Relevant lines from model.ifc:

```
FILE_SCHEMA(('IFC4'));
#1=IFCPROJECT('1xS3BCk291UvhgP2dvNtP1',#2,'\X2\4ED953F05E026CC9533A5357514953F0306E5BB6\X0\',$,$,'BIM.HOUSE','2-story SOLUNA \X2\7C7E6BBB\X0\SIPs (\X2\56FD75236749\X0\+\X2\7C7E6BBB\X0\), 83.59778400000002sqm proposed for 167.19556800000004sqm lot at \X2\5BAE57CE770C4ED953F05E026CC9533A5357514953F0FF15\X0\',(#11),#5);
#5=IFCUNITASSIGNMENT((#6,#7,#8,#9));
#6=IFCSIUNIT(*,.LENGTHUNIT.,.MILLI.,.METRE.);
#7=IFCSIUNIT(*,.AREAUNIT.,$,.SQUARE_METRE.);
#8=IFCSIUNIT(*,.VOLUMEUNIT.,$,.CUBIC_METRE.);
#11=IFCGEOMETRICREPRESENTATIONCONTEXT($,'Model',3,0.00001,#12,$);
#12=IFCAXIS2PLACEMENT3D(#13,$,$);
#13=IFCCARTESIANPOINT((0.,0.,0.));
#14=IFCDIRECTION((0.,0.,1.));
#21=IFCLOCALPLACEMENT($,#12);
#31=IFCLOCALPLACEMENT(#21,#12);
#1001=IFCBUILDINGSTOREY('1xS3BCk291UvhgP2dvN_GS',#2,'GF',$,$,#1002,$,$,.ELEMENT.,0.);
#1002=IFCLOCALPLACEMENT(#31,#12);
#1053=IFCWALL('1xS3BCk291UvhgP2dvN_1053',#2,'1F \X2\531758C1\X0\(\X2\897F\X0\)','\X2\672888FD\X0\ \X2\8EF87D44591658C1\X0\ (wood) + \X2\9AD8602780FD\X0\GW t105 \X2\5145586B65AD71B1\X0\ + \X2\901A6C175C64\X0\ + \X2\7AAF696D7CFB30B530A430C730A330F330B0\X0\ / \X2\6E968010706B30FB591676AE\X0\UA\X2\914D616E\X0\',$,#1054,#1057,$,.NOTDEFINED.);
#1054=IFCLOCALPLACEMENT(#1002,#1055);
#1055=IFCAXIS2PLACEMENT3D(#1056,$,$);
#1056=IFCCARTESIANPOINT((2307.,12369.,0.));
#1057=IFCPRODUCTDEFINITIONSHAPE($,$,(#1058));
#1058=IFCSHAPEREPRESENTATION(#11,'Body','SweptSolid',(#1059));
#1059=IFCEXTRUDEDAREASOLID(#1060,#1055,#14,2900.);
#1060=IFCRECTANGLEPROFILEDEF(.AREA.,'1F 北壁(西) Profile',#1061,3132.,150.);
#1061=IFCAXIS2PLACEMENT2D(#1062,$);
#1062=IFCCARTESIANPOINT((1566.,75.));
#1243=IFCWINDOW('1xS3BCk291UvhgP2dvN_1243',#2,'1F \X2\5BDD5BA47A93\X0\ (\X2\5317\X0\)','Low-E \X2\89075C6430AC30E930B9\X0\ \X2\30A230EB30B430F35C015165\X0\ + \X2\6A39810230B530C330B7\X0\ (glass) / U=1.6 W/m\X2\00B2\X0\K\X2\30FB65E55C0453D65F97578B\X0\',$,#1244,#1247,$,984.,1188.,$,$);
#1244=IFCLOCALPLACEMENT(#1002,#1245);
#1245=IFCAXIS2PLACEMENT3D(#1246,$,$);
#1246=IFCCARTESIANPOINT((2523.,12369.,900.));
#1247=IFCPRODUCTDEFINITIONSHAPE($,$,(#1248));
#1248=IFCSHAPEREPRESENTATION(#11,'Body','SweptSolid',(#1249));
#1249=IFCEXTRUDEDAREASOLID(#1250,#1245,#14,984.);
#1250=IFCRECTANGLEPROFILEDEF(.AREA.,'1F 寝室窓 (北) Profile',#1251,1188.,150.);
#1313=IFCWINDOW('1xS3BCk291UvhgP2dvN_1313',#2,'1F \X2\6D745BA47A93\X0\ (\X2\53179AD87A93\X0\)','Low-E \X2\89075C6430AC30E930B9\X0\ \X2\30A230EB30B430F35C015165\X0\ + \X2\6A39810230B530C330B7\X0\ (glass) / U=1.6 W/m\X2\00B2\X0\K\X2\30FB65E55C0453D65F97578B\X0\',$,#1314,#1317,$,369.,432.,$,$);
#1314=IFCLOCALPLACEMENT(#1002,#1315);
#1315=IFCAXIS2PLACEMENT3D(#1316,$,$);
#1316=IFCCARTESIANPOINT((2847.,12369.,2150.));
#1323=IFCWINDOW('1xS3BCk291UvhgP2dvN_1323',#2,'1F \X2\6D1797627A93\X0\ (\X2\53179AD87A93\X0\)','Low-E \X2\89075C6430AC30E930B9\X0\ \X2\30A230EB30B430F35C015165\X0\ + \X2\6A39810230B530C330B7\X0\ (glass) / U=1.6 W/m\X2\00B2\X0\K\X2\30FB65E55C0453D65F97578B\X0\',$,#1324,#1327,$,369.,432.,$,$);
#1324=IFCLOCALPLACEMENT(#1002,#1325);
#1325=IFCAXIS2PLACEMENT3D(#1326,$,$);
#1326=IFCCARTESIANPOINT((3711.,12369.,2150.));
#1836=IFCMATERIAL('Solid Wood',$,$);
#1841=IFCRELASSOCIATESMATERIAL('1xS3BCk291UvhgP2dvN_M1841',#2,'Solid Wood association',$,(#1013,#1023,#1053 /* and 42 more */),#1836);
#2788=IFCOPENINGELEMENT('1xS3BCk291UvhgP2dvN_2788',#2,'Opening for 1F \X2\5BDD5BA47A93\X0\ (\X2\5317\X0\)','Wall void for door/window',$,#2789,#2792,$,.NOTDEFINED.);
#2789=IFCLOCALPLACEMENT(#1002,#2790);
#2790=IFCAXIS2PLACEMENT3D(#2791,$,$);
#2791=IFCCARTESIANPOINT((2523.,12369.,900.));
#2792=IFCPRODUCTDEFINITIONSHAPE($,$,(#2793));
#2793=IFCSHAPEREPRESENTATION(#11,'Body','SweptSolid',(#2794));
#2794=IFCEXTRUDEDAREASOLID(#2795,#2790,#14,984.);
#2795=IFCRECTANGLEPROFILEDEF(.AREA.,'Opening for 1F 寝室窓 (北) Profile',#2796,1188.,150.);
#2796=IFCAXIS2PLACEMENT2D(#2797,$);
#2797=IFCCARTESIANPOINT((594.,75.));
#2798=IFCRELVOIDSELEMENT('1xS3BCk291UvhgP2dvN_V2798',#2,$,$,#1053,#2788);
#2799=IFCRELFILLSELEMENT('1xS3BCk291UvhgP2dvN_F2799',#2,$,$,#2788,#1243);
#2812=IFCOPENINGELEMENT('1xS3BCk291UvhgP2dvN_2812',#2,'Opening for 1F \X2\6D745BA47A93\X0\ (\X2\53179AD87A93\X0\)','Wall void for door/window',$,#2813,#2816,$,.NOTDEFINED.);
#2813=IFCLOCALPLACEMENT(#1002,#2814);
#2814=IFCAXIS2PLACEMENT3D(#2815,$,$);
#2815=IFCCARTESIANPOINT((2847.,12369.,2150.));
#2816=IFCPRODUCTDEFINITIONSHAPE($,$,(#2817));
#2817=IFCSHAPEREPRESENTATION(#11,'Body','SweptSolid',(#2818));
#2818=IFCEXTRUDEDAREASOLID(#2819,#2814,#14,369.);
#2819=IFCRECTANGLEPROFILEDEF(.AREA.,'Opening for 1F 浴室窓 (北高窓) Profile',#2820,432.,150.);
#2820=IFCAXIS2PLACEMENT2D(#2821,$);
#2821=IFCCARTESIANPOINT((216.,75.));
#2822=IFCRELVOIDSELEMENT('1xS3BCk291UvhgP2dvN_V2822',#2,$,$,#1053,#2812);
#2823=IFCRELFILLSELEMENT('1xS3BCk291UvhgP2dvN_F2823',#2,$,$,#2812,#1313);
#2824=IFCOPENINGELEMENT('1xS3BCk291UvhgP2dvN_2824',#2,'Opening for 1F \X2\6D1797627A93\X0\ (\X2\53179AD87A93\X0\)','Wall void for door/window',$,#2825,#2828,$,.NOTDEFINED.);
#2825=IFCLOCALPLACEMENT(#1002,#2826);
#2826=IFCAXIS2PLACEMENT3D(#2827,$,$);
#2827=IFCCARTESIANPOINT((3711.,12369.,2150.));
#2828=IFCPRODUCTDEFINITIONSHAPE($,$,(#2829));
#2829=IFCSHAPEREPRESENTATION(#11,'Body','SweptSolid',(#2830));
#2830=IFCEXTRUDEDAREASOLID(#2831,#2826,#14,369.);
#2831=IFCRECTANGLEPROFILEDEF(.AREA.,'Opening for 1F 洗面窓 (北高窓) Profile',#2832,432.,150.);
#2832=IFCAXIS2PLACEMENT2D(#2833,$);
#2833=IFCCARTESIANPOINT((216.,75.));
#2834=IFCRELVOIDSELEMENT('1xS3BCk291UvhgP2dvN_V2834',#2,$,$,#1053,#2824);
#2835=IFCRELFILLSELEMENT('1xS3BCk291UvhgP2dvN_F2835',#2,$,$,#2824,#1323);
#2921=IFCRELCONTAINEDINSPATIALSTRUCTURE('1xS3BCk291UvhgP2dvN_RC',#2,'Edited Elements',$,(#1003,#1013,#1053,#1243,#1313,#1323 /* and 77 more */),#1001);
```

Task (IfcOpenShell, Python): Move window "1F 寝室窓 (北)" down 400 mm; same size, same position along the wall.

```python
import numpy as np
import ifcopenshell
import ifcopenshell.api.geometry
import ifcopenshell.util.placement
import ifcopenshell.util.unit

model = ifcopenshell.open("model.ifc")
unit_scale = ifcopenshell.util.unit.calculate_unit_scale(model)

window = model.by_guid("1xS3BCk291UvhgP2dvN_1243")
opening = window.FillsVoids[0].RelatingOpeningElement
dz = -0.4 / unit_scale

shift = np.array([0.0, 0.0, dz])
# The window is not placed relative to its opening, so move both.
for product in (opening, window):
    matrix = ifcopenshell.util.placement.get_local_placement(product.ObjectPlacement)
    matrix[:3, 3] += shift
    ifcopenshell.api.geometry.edit_object_placement(model, product=product, matrix=matrix, is_si=False)

print(f"moved by {dz * unit_scale:+.3f} m")

model.write("model_rev.ifc")
```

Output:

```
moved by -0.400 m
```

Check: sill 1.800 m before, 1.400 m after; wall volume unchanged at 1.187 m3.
